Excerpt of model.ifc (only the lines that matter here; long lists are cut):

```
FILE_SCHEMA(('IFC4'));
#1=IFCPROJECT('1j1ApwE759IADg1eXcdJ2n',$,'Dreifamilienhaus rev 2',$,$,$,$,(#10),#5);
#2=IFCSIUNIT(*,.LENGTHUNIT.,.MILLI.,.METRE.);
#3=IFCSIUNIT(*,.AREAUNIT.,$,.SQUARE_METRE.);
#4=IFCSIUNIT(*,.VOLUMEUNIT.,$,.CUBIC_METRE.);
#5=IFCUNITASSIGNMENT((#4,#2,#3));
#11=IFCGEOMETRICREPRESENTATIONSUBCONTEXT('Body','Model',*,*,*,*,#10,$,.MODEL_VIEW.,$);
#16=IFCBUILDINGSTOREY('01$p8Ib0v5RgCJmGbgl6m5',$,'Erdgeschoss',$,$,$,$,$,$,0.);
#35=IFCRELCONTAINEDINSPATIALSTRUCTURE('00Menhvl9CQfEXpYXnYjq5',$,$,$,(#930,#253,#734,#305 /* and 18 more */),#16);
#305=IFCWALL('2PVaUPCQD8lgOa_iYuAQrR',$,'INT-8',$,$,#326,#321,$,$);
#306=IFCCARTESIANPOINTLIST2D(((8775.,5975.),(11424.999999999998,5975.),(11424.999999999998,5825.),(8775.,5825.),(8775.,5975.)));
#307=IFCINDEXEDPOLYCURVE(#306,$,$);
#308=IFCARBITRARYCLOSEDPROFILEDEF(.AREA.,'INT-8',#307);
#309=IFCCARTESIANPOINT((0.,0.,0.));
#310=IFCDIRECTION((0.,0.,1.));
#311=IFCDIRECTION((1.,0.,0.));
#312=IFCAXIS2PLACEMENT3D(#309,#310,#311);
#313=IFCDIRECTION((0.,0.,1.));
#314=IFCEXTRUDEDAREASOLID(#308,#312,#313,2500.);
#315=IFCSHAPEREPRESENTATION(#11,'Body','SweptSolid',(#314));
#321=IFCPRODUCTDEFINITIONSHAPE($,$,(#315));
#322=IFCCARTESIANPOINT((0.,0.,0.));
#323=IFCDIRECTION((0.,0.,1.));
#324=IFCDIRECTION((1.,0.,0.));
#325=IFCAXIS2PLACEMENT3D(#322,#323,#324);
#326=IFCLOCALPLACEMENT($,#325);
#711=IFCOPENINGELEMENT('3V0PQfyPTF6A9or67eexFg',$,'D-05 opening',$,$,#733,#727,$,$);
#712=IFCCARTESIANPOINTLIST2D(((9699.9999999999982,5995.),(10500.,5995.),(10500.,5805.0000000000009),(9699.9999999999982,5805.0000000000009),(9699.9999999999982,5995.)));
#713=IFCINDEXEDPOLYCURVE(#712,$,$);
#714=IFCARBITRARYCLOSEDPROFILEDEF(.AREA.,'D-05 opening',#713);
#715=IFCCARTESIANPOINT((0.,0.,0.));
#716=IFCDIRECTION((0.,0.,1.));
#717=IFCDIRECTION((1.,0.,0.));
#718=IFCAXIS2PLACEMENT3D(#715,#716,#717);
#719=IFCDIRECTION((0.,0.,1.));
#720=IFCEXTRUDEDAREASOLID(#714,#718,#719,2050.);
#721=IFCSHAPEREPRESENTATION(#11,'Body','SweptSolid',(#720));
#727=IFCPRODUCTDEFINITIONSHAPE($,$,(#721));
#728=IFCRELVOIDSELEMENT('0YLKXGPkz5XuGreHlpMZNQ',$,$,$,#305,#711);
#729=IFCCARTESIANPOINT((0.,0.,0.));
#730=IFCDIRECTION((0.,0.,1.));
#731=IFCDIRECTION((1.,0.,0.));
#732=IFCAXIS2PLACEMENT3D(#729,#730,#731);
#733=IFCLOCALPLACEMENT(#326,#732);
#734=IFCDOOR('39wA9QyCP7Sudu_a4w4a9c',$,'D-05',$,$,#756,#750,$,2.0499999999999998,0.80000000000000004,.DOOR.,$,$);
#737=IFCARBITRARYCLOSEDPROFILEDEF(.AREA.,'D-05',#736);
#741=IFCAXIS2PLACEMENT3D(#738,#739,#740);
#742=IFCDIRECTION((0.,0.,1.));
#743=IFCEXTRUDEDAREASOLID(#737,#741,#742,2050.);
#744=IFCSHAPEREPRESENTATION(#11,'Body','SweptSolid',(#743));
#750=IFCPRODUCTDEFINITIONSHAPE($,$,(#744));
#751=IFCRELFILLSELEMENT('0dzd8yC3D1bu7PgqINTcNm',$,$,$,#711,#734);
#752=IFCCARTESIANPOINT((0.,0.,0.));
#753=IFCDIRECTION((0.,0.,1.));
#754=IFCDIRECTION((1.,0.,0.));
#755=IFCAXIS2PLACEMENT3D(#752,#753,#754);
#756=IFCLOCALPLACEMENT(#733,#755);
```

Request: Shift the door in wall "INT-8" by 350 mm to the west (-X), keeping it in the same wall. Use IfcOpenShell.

```python
import ifcopenshell
import ifcopenshell.api.geometry
import ifcopenshell.util.placement

model = ifcopenshell.open("model.ifc")

door = model.by_guid("39wA9QyCP7Sudu_a4w4a9c")
opening = door.FillsVoids[0].RelatingOpeningElement
wall = opening.VoidsElements[0].RelatingBuildingElement

wall_matrix = ifcopenshell.util.placement.get_local_placement(wall.ObjectPlacement)
shift = wall_matrix[:3, 0] * -350.0
before = ifcopenshell.util.placement.get_local_placement(door.ObjectPlacement)[:3, 3].copy()

# The door is placed relative to its opening, so it follows when the opening moves.
matrix = ifcopenshell.util.placement.get_local_placement(opening.ObjectPlacement)
matrix[:3, 3] += shift
ifcopenshell.api.geometry.edit_object_placement(
    model, product=opening, matrix=matrix, is_si=False, should_transform_children=True
)

after = ifcopenshell.util.placement.get_local_placement(door.ObjectPlacement)[:3, 3]
print("door moved by", (after - before).round(3) + 0.0)

model.write("model_updated.ifc")
```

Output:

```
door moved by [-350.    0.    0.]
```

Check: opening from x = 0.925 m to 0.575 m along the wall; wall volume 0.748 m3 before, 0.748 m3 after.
